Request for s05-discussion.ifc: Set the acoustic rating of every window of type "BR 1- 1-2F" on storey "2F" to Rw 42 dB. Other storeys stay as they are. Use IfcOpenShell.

First a look at what the model holds.

```python
import ifcopenshell
import ifcopenshell.util.element

model = ifcopenshell.open("s05-discussion.ifc")
print(model.schema)
storey = next(s for s in model.by_type("IfcBuildingStorey") if s.Name == "2F")
windows = [e for e in ifcopenshell.util.element.get_decomposition(storey) if e.is_a("IfcWindow")]
seen = {}
for e in windows:
    element_type = ifcopenshell.util.element.get_type(e)
    key = (element_type.Name if element_type != e and element_type else None, ifcopenshell.util.element.get_pset(e, "Pset_WindowCommon", "AcousticRating"))
    seen[key] = seen.get(key, 0) + 1
for (name, value), count in sorted(seen.items(), key=str):
    print(count, "x", name, "|", value)
```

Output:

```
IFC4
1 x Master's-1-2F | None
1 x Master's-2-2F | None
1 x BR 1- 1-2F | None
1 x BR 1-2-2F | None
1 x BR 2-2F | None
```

```python
import ifcopenshell
import ifcopenshell.api.pset
import ifcopenshell.util.element

model = ifcopenshell.open("s05-discussion.ifc")

storey = next(s for s in model.by_type("IfcBuildingStorey") if s.Name == "2F")
windows = [e for e in ifcopenshell.util.element.get_decomposition(storey) if e.is_a("IfcWindow")]

count = 0
for e in windows:
    element_type = ifcopenshell.util.element.get_type(e)
    if element_type in (None, e) or element_type.Name != "BR 1- 1-2F":
        continue
    # add_pset returns the element's existing set when there is one.
    pset = ifcopenshell.api.pset.add_pset(model, product=e, name="Pset_WindowCommon")
    ifcopenshell.api.pset.edit_pset(model, pset=pset, properties={"AcousticRating": "Rw 42 dB"})
    count += 1

print(count, "windows updated")

model.write("s05-discussion_edited.ifc")
```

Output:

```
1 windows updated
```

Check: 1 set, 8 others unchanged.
